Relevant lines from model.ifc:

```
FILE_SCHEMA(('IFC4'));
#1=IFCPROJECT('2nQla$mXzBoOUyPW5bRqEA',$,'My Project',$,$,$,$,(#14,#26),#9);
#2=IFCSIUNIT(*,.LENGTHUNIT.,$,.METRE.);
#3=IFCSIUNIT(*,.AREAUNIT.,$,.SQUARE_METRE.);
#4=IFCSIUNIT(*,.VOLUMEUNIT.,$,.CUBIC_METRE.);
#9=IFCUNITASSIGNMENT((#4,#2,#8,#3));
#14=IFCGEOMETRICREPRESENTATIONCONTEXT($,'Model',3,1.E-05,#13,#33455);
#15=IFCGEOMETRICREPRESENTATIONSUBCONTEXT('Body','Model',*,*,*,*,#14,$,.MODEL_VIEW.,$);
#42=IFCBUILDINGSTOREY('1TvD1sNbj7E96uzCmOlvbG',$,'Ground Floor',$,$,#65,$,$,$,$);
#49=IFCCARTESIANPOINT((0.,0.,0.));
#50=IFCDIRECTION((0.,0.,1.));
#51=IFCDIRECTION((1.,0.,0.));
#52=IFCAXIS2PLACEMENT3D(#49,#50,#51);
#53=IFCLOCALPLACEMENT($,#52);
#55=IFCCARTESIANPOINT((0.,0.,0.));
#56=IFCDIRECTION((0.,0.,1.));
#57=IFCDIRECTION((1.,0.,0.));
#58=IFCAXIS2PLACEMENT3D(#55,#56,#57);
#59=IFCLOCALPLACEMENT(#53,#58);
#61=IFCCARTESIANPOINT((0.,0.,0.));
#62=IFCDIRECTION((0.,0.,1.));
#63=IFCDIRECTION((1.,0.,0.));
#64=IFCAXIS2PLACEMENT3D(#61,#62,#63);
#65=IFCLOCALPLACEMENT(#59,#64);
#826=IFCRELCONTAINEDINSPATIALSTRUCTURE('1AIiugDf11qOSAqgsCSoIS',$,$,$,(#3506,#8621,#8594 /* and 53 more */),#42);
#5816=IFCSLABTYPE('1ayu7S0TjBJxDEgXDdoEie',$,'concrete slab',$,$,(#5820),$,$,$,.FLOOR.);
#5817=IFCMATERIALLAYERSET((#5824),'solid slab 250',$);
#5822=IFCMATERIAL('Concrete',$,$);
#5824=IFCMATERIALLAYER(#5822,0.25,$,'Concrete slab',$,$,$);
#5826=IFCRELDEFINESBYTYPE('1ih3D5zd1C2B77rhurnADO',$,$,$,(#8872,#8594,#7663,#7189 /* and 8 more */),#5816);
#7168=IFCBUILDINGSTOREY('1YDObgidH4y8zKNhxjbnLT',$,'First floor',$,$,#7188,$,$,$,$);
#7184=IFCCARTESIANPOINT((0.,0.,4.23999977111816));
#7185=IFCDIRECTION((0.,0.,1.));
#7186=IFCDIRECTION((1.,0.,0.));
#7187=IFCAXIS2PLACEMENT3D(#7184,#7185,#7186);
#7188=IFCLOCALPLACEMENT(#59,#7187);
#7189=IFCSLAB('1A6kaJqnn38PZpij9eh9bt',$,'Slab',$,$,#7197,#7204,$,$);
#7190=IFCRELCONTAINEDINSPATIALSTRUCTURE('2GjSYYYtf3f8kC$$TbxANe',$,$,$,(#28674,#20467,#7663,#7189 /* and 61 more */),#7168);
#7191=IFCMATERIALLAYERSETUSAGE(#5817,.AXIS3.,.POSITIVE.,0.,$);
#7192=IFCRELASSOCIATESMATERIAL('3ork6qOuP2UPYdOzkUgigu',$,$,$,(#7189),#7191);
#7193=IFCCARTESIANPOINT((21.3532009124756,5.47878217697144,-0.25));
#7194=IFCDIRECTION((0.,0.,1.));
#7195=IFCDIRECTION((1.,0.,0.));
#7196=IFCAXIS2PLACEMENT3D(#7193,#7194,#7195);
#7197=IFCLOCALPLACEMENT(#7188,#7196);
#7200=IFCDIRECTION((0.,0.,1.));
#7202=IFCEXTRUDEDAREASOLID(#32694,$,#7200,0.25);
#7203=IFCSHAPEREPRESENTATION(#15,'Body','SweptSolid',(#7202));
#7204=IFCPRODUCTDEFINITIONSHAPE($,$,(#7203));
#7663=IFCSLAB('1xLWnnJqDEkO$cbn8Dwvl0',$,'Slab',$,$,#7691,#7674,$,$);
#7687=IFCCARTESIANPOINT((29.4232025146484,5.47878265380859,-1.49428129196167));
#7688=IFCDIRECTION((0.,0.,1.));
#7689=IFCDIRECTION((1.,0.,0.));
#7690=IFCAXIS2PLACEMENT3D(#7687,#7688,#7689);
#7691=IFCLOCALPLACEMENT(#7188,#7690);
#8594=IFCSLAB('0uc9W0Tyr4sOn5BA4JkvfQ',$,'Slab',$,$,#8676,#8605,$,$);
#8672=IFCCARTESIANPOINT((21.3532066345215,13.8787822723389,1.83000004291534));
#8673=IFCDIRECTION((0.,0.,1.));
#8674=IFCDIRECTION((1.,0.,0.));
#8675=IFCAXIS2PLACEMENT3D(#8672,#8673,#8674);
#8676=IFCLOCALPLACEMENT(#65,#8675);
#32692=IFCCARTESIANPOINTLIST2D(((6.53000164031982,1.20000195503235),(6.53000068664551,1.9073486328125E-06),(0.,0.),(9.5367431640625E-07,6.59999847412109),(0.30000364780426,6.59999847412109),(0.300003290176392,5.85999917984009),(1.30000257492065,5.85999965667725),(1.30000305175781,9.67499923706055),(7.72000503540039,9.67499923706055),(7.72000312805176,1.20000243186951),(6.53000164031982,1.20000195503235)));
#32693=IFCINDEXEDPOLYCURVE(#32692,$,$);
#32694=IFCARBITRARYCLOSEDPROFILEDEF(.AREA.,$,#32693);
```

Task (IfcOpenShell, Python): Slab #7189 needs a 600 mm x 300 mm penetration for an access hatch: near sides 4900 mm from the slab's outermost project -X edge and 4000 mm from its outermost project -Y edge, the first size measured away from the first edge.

```python
import numpy as np
import ifcopenshell
import ifcopenshell.api.feature
import ifcopenshell.api.geometry
import ifcopenshell.api.root
import ifcopenshell.geom
import ifcopenshell.util.placement
import ifcopenshell.util.representation
import ifcopenshell.util.shape
import ifcopenshell.util.unit

model = ifcopenshell.open("model.ifc")
unit_scale = ifcopenshell.util.unit.calculate_unit_scale(model)
settings = ifcopenshell.geom.settings()


def volume(element):
    """Net volume in cubic metres, openings subtracted."""
    shape = ifcopenshell.geom.create_shape(settings, element)
    return ifcopenshell.util.shape.get_volume(shape.geometry)


slab = model.by_guid("1A6kaJqnn38PZpij9eh9bt")
before = volume(slab)

# Extent in the slab's own axes, in metres. The edges named are its -X and -Y sides.
slab_shape = ifcopenshell.geom.create_shape(settings, slab)
vertices = ifcopenshell.util.shape.get_vertices(slab_shape.geometry)
x_min, y_min, bottom = vertices.min(axis=0)
top = vertices[:, 2].max()

opening = ifcopenshell.api.root.create_entity(model, ifc_class="IfcOpeningElement", name="Access hatch opening", predefined_type="OPENING")
context = ifcopenshell.util.representation.get_context(model, "Model", "Body", "MODEL_VIEW")
width, depth = 0.6, 0.3
outline = [(0.0, 0.0), (width, 0.0), (width, depth), (0.0, depth), (0.0, 0.0)]
# Overshoot both faces by 50 mm so the cut is clean.
shape = ifcopenshell.api.geometry.add_slab_representation(
    model, context=context, depth=top - bottom + 0.1, polyline=outline
)
ifcopenshell.api.geometry.assign_representation(model, product=opening, representation=shape)

matrix = ifcopenshell.util.placement.get_local_placement(slab.ObjectPlacement)
matrix[:, 3] = matrix @ np.append(np.array([x_min + 4.9, y_min + 4, bottom - 0.05]) / unit_scale, 1.0)
ifcopenshell.api.geometry.edit_object_placement(model, product=opening, matrix=matrix, is_si=False)
ifcopenshell.api.feature.add_feature(model, feature=opening, element=slab)

after = volume(slab)

print(f"slab volume {before:.3f} -> {after:.3f} m3")

model.write("model_v2.ifc")
```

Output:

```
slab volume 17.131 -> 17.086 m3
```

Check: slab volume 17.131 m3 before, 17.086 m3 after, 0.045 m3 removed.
